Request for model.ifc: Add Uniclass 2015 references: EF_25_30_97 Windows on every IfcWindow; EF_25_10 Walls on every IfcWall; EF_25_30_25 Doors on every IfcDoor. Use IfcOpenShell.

First a look at what the model holds.

```python
import ifcopenshell

model = ifcopenshell.open("model.ifc")
print(model.schema)
print("classifications:", [c.Name for c in model.by_type("IfcClassification")])
for ifc_class in ("IfcDoor", "IfcRoof", "IfcStair", "IfcWall", "IfcWindow"):
    print(ifc_class, len(model.by_type(ifc_class)))
```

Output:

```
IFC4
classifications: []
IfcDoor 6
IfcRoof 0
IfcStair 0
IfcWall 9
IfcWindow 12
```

```python
import ifcopenshell
import ifcopenshell.api.classification

model = ifcopenshell.open("model.ifc")

system = ifcopenshell.api.classification.add_classification(model, classification="Uniclass 2015")

codes = {
    "IfcWindow": ("EF_25_30_97", "Windows"),
    "IfcWall": ("EF_25_10", "Walls"),
    "IfcDoor": ("EF_25_30_25", "Doors"),
}
for ifc_class, (code, name) in codes.items():
    products = model.by_type(ifc_class)
    ifcopenshell.api.classification.add_reference(
        model, products=products, classification=system, identification=code, name=name
    )
    print(code, len(products))

model.write("model_v2.ifc")
```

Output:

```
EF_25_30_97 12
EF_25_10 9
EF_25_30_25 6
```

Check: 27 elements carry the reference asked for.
